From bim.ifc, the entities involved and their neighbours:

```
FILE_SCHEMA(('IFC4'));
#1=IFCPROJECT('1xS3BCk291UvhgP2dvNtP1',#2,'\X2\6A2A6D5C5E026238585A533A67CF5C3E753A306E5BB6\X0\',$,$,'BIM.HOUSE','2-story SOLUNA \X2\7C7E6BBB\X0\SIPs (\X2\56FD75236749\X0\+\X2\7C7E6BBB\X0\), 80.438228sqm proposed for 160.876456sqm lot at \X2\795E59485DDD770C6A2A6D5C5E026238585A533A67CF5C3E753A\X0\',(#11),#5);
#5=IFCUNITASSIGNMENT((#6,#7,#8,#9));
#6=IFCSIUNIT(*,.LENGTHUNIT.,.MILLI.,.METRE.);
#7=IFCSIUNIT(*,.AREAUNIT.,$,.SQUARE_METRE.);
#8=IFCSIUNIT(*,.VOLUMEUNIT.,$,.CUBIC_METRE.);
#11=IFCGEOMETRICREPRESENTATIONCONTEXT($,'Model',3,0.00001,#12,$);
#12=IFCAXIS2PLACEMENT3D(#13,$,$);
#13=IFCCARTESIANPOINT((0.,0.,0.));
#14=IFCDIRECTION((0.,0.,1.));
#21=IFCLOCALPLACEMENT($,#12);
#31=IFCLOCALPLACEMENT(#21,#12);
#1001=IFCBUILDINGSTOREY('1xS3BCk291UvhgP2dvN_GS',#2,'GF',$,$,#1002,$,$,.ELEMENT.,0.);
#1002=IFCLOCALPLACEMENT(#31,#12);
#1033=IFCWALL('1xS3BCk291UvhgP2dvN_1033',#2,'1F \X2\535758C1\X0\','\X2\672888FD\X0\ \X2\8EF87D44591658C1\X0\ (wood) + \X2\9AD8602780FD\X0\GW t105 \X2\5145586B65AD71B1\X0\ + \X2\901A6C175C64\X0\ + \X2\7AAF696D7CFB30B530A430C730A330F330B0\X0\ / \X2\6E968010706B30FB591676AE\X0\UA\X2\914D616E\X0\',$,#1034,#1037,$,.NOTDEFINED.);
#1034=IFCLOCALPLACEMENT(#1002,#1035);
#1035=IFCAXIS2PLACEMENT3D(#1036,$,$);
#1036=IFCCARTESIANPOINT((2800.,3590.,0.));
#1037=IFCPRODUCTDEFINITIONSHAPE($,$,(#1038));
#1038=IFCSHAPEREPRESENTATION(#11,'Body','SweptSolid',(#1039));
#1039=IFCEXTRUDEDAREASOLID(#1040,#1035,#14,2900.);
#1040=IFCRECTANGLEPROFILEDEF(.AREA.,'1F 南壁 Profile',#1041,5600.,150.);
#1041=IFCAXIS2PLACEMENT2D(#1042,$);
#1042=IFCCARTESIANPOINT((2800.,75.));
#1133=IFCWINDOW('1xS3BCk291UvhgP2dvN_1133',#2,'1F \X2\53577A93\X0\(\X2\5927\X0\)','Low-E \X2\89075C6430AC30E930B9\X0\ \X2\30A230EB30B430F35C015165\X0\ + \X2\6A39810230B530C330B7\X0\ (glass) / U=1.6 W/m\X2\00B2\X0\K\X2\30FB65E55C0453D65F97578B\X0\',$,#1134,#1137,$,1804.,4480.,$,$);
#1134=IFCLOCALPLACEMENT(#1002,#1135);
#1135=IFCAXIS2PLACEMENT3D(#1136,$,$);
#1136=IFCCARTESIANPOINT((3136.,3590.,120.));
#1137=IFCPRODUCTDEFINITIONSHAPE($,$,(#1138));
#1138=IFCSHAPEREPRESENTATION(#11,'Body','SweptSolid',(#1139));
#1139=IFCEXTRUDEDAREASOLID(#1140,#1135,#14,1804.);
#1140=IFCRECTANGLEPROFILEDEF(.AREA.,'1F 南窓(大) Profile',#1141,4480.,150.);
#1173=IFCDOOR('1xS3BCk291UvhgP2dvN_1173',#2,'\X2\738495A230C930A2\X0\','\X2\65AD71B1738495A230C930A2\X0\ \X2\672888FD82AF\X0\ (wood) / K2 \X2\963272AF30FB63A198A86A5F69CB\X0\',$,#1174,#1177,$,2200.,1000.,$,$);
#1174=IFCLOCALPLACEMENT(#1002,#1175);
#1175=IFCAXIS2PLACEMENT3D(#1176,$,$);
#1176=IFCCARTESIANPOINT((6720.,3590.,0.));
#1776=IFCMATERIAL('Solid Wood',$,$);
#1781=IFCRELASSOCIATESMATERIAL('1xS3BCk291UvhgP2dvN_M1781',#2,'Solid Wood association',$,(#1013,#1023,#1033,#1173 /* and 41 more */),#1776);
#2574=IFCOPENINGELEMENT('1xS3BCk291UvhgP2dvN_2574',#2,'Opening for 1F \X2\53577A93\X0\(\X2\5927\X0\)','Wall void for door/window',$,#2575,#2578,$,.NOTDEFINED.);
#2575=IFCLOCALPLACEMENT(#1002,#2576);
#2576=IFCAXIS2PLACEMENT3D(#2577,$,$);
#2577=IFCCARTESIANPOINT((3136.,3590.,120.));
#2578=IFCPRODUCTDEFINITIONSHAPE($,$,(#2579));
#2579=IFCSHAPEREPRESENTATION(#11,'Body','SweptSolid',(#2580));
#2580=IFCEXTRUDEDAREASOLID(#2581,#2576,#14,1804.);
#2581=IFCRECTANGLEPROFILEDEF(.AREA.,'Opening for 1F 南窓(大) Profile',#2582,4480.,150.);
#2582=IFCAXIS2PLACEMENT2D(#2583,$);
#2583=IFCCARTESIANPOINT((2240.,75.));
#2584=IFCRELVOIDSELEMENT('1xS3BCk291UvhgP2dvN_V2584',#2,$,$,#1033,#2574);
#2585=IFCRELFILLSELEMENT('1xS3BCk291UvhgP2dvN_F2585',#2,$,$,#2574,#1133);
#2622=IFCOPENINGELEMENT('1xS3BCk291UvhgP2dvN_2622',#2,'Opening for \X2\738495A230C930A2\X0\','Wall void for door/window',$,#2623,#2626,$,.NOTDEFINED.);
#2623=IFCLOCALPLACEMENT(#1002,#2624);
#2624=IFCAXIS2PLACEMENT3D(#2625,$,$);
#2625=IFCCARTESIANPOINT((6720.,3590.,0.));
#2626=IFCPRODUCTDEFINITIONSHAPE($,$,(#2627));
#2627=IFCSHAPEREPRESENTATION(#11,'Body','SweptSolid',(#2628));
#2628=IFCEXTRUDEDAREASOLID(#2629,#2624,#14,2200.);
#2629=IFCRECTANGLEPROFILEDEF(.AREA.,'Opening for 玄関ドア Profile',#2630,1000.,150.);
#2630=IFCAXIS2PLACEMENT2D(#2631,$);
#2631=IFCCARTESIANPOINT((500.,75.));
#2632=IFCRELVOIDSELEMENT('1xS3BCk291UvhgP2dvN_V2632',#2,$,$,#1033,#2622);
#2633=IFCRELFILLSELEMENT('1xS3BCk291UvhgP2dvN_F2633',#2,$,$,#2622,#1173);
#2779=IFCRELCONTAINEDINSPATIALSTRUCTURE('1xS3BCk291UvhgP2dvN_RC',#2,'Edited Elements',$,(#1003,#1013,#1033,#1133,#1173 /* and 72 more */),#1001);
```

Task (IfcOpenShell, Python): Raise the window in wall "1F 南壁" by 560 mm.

```python
import numpy as np
import ifcopenshell
import ifcopenshell.api.geometry
import ifcopenshell.util.placement
import ifcopenshell.util.unit

model = ifcopenshell.open("bim.ifc")
unit_scale = ifcopenshell.util.unit.calculate_unit_scale(model)

window = model.by_id(1133)
opening = window.FillsVoids[0].RelatingOpeningElement
dz = 560.0

shift = np.array([0.0, 0.0, dz])
# The window is not placed relative to its opening, so move both.
for product in (opening, window):
    matrix = ifcopenshell.util.placement.get_local_placement(product.ObjectPlacement)
    matrix[:3, 3] += shift
    ifcopenshell.api.geometry.edit_object_placement(model, product=product, matrix=matrix, is_si=False)

print(f"moved by {dz * unit_scale:+.3f} m")

model.write("bim-out.ifc")
```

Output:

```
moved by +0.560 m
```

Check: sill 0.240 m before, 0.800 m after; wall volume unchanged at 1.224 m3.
